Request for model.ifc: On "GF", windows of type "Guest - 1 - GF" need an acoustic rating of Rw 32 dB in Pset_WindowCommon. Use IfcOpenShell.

First a look at what the model holds.

```python
import ifcopenshell
import ifcopenshell.util.element

model = ifcopenshell.open("model.ifc")
print(model.schema)
storey = next(s for s in model.by_type("IfcBuildingStorey") if s.Name == "GF")
windows = [e for e in ifcopenshell.util.element.get_decomposition(storey) if e.is_a("IfcWindow")]
seen = {}
for e in windows:
    element_type = ifcopenshell.util.element.get_type(e)
    key = (element_type.Name if element_type != e and element_type else None, ifcopenshell.util.element.get_pset(e, "Pset_WindowCommon", "AcousticRating"))
    seen[key] = seen.get(key, 0) + 1
for (name, value), count in sorted(seen.items(), key=str):
    print(count, "x", name, "|", value)
```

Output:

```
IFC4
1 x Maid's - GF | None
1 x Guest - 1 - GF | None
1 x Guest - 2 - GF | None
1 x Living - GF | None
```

```python
import ifcopenshell
import ifcopenshell.api.pset
import ifcopenshell.util.element

model = ifcopenshell.open("model.ifc")

storey = next(s for s in model.by_type("IfcBuildingStorey") if s.Name == "GF")
windows = [e for e in ifcopenshell.util.element.get_decomposition(storey) if e.is_a("IfcWindow")]

count = 0
for e in windows:
    element_type = ifcopenshell.util.element.get_type(e)
    if element_type in (None, e) or element_type.Name != "Guest - 1 - GF":
        continue
    # add_pset returns the element's existing set when there is one.
    pset = ifcopenshell.api.pset.add_pset(model, product=e, name="Pset_WindowCommon")
    ifcopenshell.api.pset.edit_pset(model, pset=pset, properties={"AcousticRating": "Rw 32 dB"})
    count += 1

print(count, "windows updated")

model.write("model-out.ifc")
```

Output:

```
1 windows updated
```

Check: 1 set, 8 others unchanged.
